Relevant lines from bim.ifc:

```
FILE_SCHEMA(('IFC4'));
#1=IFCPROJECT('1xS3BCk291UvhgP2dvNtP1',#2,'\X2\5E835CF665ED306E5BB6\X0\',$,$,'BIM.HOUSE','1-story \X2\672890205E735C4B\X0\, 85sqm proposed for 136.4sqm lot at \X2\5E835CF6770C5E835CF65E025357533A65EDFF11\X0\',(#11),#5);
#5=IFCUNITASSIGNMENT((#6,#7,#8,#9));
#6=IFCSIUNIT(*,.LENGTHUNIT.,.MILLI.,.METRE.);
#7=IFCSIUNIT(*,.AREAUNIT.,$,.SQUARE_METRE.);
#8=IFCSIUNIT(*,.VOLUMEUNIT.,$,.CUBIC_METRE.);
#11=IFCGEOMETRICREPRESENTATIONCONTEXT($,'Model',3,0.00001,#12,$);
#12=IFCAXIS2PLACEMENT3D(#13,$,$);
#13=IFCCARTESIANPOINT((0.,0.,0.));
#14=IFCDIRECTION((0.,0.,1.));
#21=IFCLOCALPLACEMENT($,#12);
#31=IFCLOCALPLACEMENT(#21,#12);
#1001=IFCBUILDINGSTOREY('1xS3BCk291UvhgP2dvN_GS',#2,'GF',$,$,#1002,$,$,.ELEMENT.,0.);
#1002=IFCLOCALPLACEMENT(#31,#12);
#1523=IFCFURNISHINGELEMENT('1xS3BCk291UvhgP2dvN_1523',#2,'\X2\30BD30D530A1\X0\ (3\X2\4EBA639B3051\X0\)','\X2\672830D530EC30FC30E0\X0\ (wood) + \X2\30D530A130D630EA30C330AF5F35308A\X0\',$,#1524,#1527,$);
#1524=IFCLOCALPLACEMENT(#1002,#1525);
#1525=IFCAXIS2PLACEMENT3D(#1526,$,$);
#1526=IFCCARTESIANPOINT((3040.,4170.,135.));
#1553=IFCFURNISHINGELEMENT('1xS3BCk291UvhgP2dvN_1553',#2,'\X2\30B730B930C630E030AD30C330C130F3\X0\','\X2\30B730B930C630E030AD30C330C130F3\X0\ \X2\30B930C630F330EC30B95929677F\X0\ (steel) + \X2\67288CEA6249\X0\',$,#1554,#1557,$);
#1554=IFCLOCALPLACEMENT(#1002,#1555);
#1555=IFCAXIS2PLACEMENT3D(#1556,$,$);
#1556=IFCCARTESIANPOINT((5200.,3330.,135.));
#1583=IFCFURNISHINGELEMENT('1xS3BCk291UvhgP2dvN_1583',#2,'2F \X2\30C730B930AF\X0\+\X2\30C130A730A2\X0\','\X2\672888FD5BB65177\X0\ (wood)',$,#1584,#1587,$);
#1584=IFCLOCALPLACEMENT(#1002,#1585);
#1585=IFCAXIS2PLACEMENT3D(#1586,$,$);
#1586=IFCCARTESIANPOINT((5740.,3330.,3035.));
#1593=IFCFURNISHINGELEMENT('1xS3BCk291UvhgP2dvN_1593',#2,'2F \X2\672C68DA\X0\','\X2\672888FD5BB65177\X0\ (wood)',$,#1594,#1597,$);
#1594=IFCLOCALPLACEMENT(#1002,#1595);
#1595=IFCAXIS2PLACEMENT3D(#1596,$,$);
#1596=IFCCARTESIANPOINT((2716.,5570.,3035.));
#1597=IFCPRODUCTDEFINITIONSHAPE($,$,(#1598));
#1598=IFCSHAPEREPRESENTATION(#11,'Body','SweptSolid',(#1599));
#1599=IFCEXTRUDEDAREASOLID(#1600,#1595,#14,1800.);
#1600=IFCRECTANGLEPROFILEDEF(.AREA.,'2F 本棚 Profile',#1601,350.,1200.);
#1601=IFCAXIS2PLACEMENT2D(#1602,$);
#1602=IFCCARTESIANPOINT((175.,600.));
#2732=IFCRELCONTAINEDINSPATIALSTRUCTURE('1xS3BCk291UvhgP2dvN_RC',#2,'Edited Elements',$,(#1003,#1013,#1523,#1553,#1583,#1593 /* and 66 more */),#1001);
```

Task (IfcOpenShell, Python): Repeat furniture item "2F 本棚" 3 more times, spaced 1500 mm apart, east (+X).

```python
import numpy as np
import ifcopenshell
import ifcopenshell.api.geometry
import ifcopenshell.api.root
import ifcopenshell.util.element
import ifcopenshell.util.placement
import ifcopenshell.util.unit

model = ifcopenshell.open("bim.ifc")
unit_scale = ifcopenshell.util.unit.calculate_unit_scale(model)


def reuse_history(source, copy):
    """copy_class also copies each property set's owner history, people and application; keep the originals."""
    for rel in copy.IsDefinedBy:
        if rel.is_a("IfcRelDefinesByProperties") and (history := rel.RelatingPropertyDefinition.OwnerHistory):
            rel.RelatingPropertyDefinition.OwnerHistory = source.OwnerHistory
            ifcopenshell.util.element.remove_deep2(model, history)


source = model.by_id(1593)
base = ifcopenshell.util.placement.get_local_placement(source.ObjectPlacement)
step = np.array([1.0, 0.0, 0.0]) * 1.5 / unit_scale

for i in range(1, 4):
    copy = ifcopenshell.api.root.copy_class(model, product=source)
    copy.Representation = ifcopenshell.util.element.copy_deep(
        model, source.Representation, exclude=["IfcGeometricRepresentationContext", "IfcRepresentationMap"]
    )
    reuse_history(source, copy)
    matrix = base.copy()
    matrix[:3, 3] += i * step
    print("added at", matrix[:3, 3].round(3) + 0.0)
    ifcopenshell.api.geometry.edit_object_placement(model, product=copy, matrix=matrix, is_si=False)

model.write("bim-out.ifc")
```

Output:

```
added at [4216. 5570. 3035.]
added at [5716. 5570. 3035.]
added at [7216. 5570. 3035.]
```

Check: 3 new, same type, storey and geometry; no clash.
